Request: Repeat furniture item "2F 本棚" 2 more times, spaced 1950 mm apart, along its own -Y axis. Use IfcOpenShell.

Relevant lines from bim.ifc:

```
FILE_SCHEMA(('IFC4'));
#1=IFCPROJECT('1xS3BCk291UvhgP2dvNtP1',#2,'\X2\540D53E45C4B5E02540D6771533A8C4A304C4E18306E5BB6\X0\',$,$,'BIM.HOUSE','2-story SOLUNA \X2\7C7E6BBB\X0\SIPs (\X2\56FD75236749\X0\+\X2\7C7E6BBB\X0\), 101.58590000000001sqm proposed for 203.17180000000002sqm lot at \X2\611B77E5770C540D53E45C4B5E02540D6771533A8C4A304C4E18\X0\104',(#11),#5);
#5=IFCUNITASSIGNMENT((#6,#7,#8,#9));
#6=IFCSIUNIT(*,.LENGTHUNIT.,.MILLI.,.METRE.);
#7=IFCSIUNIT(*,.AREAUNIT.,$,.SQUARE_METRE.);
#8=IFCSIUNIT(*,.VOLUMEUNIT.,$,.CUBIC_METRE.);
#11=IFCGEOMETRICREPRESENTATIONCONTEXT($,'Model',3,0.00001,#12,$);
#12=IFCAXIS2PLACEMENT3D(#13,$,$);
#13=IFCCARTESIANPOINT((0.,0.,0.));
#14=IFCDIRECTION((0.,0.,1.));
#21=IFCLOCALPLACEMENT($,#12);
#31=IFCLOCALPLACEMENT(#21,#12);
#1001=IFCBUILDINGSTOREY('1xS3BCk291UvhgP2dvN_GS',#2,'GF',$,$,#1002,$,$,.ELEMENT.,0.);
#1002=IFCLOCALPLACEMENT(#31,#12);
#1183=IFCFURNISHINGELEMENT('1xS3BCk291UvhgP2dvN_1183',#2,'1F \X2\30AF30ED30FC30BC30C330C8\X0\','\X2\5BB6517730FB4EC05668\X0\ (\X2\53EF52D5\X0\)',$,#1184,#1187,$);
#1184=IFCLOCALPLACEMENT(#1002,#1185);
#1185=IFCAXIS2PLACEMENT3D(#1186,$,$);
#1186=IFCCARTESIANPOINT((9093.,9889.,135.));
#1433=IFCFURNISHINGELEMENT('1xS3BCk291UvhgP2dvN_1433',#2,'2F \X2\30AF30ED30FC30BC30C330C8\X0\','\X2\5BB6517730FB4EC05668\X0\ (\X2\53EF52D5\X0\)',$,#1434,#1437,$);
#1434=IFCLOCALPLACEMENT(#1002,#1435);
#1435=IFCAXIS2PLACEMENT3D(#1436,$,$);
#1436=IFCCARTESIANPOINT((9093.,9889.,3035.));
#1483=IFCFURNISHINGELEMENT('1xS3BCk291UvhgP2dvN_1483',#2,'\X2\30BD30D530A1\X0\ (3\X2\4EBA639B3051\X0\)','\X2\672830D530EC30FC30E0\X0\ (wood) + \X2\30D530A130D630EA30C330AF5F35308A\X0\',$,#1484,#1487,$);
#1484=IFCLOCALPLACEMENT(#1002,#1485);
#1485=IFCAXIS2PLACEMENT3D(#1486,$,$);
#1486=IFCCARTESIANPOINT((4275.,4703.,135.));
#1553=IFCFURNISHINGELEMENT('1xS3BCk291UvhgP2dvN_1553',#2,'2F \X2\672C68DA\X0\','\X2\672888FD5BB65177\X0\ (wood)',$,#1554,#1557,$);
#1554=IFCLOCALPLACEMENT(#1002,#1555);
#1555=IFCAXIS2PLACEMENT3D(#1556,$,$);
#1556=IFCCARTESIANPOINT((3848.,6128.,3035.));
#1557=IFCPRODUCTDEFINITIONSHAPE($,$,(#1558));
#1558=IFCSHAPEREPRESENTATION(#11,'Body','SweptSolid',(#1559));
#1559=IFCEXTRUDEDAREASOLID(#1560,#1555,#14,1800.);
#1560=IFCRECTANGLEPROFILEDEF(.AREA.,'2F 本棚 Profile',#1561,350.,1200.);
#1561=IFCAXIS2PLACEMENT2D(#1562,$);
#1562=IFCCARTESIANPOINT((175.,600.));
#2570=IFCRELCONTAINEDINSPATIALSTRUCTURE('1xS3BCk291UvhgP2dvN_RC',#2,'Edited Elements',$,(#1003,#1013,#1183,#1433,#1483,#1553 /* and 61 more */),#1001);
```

```python
import ifcopenshell
import ifcopenshell.api.geometry
import ifcopenshell.api.root
import ifcopenshell.util.element
import ifcopenshell.util.placement
import ifcopenshell.util.unit

model = ifcopenshell.open("bim.ifc")
unit_scale = ifcopenshell.util.unit.calculate_unit_scale(model)


def reuse_history(source, copy):
    """copy_class also copies each property set's owner history, people and application; keep the originals."""
    for rel in copy.IsDefinedBy:
        if rel.is_a("IfcRelDefinesByProperties") and (history := rel.RelatingPropertyDefinition.OwnerHistory):
            rel.RelatingPropertyDefinition.OwnerHistory = source.OwnerHistory
            ifcopenshell.util.element.remove_deep2(model, history)


source = model.by_guid("1xS3BCk291UvhgP2dvN_1553")
base = ifcopenshell.util.placement.get_local_placement(source.ObjectPlacement)
step = -base[:3, 1] * 1.95 / unit_scale

for i in range(1, 3):
    copy = ifcopenshell.api.root.copy_class(model, product=source)
    copy.Representation = ifcopenshell.util.element.copy_deep(
        model, source.Representation, exclude=["IfcGeometricRepresentationContext", "IfcRepresentationMap"]
    )
    reuse_history(source, copy)
    matrix = base.copy()
    matrix[:3, 3] += i * step
    print("added at", matrix[:3, 3].round(3) + 0.0)
    ifcopenshell.api.geometry.edit_object_placement(model, product=copy, matrix=matrix, is_si=False)

model.write("bim_v2.ifc")
```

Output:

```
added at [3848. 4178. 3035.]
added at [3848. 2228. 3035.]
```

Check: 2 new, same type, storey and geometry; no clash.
